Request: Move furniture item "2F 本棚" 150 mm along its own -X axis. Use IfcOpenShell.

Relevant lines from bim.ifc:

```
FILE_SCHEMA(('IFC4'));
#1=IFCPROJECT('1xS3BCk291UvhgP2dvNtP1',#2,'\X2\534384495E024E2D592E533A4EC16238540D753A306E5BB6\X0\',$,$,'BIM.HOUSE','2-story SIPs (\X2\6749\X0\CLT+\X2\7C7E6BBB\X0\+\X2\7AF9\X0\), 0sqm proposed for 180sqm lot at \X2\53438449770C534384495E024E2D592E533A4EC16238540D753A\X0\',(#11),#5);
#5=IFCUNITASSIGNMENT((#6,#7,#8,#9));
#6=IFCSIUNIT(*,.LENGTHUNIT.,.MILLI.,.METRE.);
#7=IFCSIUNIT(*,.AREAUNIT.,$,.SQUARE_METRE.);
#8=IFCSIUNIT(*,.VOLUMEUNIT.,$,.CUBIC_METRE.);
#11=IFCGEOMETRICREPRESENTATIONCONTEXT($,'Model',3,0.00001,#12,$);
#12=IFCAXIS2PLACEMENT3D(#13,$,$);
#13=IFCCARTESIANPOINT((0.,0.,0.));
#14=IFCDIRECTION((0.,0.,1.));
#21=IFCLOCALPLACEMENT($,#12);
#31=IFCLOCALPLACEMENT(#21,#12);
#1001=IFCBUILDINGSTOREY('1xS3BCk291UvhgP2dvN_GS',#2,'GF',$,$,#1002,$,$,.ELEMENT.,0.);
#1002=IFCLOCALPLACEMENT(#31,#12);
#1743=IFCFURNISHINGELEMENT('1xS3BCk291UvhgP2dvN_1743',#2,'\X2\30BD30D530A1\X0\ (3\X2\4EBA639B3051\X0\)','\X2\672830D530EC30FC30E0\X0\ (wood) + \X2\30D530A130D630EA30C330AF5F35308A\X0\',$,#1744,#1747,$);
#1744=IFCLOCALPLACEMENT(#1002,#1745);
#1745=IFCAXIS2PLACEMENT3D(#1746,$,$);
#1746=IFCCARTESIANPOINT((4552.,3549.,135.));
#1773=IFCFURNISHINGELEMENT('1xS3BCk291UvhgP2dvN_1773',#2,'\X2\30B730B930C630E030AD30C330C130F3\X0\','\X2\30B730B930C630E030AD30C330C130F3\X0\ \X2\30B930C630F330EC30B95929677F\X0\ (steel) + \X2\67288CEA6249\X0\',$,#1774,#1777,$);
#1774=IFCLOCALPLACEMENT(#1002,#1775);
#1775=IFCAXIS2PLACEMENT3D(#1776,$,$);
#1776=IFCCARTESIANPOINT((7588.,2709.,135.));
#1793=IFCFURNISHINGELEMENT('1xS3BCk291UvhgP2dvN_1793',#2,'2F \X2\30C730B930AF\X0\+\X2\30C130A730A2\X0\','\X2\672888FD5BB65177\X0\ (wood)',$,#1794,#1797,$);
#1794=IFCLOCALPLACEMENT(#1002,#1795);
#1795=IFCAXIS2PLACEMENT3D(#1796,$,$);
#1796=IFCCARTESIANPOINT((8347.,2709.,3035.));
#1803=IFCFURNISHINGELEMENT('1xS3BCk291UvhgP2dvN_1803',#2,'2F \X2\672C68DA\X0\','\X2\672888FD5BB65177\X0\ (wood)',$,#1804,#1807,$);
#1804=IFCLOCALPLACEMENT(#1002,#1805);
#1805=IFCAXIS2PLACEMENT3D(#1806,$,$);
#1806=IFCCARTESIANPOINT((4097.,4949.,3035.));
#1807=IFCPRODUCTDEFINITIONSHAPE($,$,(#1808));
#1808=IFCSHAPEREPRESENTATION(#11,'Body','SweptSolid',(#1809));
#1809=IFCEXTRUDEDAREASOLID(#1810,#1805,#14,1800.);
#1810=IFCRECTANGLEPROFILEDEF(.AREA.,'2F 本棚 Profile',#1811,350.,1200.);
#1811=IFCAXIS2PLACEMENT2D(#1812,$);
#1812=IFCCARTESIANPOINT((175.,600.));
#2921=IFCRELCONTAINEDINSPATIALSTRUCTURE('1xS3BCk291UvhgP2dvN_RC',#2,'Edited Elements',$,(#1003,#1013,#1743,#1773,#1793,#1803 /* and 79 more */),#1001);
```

```python
import ifcopenshell
import ifcopenshell.api.geometry
import ifcopenshell.util.placement

model = ifcopenshell.open("bim.ifc")

item = model.by_id(1803)
matrix = ifcopenshell.util.placement.get_local_placement(item.ObjectPlacement)
matrix[:3, 3] -= matrix[:3, 0] * 150.0
ifcopenshell.api.geometry.edit_object_placement(model, product=item, matrix=matrix, is_si=False)

print(ifcopenshell.util.placement.get_local_placement(item.ObjectPlacement).round(3) + 0.0)

model.write("bim_updated.ifc")
```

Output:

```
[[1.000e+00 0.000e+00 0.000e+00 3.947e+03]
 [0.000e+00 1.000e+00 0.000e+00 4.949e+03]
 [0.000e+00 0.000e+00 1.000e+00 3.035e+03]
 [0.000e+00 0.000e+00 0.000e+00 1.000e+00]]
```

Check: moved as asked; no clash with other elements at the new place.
